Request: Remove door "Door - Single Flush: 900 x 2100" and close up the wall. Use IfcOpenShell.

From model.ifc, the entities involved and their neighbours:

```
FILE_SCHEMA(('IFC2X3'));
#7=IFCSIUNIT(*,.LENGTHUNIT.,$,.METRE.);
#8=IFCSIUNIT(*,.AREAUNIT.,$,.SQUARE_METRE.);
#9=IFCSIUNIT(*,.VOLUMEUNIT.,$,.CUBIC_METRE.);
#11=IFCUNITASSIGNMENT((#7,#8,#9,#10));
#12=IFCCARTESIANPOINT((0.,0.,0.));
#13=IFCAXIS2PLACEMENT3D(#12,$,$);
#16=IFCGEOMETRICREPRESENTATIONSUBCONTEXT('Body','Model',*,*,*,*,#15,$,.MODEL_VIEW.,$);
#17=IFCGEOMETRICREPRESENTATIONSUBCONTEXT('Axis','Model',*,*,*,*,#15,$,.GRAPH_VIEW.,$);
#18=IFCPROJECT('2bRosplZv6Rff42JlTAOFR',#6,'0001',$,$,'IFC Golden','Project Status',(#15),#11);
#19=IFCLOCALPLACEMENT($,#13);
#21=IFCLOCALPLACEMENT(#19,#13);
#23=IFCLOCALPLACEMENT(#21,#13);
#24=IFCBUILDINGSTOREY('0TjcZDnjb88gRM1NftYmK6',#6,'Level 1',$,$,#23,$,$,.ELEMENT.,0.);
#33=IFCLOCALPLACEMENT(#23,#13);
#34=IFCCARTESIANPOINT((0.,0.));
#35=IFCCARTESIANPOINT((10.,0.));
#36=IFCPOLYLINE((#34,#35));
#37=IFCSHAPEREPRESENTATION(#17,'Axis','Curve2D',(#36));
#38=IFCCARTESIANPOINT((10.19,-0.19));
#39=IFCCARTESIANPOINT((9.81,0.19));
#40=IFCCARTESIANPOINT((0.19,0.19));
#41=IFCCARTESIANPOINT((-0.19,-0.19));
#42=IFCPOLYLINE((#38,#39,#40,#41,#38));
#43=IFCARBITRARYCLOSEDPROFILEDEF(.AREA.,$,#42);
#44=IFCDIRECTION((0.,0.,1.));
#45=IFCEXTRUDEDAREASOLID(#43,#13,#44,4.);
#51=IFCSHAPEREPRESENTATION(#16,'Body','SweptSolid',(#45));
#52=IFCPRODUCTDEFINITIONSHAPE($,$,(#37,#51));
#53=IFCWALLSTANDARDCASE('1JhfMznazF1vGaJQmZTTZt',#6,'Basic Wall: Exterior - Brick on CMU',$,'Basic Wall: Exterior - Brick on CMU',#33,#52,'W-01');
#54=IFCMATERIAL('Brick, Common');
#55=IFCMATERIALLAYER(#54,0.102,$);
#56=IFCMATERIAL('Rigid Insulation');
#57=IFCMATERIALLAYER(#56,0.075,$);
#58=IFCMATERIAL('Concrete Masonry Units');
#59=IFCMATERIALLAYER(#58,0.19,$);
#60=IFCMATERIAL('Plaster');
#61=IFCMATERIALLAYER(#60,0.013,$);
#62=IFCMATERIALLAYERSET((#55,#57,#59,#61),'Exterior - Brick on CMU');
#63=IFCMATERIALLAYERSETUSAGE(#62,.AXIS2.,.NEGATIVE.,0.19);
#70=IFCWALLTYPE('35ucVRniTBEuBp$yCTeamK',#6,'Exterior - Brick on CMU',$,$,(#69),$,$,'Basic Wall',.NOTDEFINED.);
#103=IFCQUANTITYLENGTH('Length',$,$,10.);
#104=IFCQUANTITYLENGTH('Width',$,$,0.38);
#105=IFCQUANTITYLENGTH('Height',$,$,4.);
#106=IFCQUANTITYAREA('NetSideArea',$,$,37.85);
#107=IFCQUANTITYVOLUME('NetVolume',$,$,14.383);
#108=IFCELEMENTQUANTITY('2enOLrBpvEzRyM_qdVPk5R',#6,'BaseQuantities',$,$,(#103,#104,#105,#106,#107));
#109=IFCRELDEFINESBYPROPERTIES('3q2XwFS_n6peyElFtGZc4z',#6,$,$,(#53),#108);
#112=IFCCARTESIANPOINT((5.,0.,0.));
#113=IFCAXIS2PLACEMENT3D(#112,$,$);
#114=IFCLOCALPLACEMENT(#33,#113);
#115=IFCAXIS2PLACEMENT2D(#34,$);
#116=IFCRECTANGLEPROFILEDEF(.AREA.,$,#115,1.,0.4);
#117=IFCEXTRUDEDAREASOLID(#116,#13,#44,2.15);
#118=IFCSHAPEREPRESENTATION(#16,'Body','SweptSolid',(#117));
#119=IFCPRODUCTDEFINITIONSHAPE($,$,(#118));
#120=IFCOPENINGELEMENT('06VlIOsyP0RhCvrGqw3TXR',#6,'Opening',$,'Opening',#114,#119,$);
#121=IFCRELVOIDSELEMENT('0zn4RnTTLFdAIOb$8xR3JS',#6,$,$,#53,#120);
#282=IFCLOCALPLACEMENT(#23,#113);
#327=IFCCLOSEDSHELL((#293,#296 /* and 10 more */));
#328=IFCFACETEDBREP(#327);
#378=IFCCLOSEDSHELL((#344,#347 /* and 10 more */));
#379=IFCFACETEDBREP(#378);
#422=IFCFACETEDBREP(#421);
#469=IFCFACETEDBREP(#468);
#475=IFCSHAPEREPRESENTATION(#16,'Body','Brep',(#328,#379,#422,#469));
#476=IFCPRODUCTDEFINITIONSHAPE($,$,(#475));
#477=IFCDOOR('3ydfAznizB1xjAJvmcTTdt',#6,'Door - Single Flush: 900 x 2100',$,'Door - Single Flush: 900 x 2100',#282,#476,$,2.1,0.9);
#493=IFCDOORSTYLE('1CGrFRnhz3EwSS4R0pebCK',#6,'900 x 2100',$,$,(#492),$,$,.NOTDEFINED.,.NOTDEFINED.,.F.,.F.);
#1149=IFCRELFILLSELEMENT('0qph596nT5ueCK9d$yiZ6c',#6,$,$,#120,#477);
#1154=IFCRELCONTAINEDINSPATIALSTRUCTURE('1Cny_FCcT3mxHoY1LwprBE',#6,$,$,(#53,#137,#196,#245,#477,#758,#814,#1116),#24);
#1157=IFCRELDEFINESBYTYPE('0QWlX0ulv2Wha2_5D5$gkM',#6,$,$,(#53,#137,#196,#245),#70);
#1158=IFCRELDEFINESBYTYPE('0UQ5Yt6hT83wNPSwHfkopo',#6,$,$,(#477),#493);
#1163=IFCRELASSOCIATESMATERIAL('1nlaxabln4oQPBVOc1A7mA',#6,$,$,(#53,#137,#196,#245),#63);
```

```python
import ifcopenshell
import ifcopenshell.api.feature
import ifcopenshell.api.pset
import ifcopenshell.api.root
import ifcopenshell.geom
import ifcopenshell.util.element
import ifcopenshell.util.shape
import ifcopenshell.util.unit

model = ifcopenshell.open("model.ifc")
area_scale = ifcopenshell.util.unit.calculate_unit_scale(model, "AREAUNIT")
volume_scale = ifcopenshell.util.unit.calculate_unit_scale(model, "VOLUMEUNIT")
settings = ifcopenshell.geom.settings()


def volume(element):
    """Net volume in cubic metres, openings subtracted."""
    shape = ifcopenshell.geom.create_shape(settings, element)
    return ifcopenshell.util.shape.get_volume(shape.geometry)


door = model.by_guid("3ydfAznizB1xjAJvmcTTdt")
opening = door.FillsVoids[0].RelatingOpeningElement
wall = opening.VoidsElements[0].RelatingBuildingElement
before = volume(wall)

ifcopenshell.api.root.remove_product(model, product=door)
ifcopenshell.api.feature.remove_feature(model, feature=opening)

after = volume(wall)
thickness = 0.38  # wall thickness in metres

# Update the wall's stored quantities.
qto = model.by_id(ifcopenshell.util.element.get_pset(wall, "BaseQuantities", should_inherit=False)["id"])
ifcopenshell.api.pset.edit_qto(model, qto=qto, properties={
    "NetSideArea": after / thickness / area_scale,
    "NetVolume": after / volume_scale,
})

print(f"wall volume {before:.3f} -> {after:.3f} m3")

model.write("model_rev.ifc")
```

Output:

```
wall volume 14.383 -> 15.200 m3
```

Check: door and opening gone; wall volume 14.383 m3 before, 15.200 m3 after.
